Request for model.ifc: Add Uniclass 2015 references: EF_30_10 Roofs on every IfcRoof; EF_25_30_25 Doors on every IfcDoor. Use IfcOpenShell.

First a look at what the model holds.

```python
import ifcopenshell

model = ifcopenshell.open("model.ifc")
print(model.schema)
print("classifications:", [c.Name for c in model.by_type("IfcClassification")])
for ifc_class in ("IfcDoor", "IfcRoof", "IfcStair", "IfcWall", "IfcWindow"):
    print(ifc_class, len(model.by_type(ifc_class)))
```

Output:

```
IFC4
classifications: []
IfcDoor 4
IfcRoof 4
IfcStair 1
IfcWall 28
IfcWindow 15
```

```python
import ifcopenshell
import ifcopenshell.api.classification

model = ifcopenshell.open("model.ifc")

system = ifcopenshell.api.classification.add_classification(model, classification="Uniclass 2015")

codes = {
    "IfcRoof": ("EF_30_10", "Roofs"),
    "IfcDoor": ("EF_25_30_25", "Doors"),
}
for ifc_class, (code, name) in codes.items():
    products = model.by_type(ifc_class)
    ifcopenshell.api.classification.add_reference(
        model, products=products, classification=system, identification=code, name=name
    )
    print(code, len(products))

model.write("model-out.ifc")
```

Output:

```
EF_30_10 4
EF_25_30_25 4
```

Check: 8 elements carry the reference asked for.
